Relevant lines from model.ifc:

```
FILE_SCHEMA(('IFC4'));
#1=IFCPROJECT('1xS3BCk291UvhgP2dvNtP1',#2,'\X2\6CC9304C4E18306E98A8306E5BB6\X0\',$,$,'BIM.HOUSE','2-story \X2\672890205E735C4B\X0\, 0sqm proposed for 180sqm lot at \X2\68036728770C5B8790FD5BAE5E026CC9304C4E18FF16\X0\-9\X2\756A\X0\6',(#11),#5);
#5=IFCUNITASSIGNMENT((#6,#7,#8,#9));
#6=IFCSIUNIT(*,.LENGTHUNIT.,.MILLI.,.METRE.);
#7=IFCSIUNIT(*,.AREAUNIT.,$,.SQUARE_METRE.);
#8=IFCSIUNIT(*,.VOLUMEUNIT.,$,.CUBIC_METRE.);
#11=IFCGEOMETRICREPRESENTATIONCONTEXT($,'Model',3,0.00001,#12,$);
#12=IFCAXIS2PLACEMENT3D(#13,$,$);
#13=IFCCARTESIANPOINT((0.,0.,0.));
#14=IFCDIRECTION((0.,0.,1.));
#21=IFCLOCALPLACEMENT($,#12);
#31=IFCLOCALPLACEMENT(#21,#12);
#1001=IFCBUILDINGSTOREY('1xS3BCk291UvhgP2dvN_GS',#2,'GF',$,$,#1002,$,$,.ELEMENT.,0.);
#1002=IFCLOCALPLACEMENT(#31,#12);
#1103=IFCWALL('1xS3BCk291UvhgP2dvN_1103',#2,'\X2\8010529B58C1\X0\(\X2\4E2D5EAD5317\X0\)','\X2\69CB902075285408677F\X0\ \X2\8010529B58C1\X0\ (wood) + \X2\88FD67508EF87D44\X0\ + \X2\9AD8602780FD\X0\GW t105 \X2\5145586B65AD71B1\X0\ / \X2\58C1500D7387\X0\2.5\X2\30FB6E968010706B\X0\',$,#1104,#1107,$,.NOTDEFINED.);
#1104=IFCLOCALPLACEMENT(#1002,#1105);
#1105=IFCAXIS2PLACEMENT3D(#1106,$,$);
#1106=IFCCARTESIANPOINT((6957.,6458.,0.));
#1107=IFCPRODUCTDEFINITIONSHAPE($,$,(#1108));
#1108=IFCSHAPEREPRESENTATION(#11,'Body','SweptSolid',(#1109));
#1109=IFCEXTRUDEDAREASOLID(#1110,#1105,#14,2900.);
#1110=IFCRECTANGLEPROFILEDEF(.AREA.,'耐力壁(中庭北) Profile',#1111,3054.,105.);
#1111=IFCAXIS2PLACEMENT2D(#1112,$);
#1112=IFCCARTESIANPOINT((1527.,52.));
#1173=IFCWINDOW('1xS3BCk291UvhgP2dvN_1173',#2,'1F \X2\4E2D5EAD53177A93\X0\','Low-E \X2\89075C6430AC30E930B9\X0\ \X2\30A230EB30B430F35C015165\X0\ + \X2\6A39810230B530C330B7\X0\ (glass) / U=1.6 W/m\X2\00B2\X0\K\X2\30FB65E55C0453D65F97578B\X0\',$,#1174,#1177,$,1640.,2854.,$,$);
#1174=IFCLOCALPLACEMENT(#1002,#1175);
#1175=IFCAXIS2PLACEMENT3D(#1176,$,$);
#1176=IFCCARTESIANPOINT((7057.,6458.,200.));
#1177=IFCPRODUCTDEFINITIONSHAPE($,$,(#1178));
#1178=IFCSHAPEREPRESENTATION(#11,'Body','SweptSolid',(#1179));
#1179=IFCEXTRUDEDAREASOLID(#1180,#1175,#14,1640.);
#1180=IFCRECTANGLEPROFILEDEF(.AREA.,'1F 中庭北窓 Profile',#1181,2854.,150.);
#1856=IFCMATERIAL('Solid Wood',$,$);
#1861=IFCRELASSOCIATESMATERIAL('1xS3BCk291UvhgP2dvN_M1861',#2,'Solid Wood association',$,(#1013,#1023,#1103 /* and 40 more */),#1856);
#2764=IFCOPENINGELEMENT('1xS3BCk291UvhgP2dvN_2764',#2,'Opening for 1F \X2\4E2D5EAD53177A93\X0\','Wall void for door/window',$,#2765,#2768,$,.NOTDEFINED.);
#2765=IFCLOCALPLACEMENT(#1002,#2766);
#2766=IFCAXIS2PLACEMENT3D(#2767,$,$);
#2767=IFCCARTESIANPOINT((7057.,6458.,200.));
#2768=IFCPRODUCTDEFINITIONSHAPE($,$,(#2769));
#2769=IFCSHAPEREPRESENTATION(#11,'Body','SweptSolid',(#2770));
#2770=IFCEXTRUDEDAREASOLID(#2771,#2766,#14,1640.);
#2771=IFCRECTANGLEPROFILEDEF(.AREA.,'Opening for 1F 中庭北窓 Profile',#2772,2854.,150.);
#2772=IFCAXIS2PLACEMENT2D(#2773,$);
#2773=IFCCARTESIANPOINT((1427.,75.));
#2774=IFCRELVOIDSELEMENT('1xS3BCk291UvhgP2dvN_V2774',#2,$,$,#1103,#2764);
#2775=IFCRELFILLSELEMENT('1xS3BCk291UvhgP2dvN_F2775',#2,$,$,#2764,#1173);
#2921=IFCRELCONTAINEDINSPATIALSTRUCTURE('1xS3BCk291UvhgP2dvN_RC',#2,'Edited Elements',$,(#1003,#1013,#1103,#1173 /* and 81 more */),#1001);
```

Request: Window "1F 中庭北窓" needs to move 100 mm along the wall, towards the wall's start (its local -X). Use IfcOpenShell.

```python
import ifcopenshell
import ifcopenshell.api.geometry
import ifcopenshell.util.placement
import ifcopenshell.util.unit

model = ifcopenshell.open("model.ifc")
unit_scale = ifcopenshell.util.unit.calculate_unit_scale(model)

window = model.by_guid("1xS3BCk291UvhgP2dvN_1173")
opening = window.FillsVoids[0].RelatingOpeningElement
wall = opening.VoidsElements[0].RelatingBuildingElement

wall_matrix = ifcopenshell.util.placement.get_local_placement(wall.ObjectPlacement)
shift = wall_matrix[:3, 0] * -0.1 / unit_scale
before = ifcopenshell.util.placement.get_local_placement(window.ObjectPlacement)[:3, 3].copy()

# The window is not placed relative to its opening, so move both.
for product in (opening, window):
    matrix = ifcopenshell.util.placement.get_local_placement(product.ObjectPlacement)
    matrix[:3, 3] += shift
    ifcopenshell.api.geometry.edit_object_placement(model, product=product, matrix=matrix, is_si=False)

after = ifcopenshell.util.placement.get_local_placement(window.ObjectPlacement)[:3, 3]
print("window moved by", (after - before).round(3) + 0.0)

model.write("model_v2.ifc")
```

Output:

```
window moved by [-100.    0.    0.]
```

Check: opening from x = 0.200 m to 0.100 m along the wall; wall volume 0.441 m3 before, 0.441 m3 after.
